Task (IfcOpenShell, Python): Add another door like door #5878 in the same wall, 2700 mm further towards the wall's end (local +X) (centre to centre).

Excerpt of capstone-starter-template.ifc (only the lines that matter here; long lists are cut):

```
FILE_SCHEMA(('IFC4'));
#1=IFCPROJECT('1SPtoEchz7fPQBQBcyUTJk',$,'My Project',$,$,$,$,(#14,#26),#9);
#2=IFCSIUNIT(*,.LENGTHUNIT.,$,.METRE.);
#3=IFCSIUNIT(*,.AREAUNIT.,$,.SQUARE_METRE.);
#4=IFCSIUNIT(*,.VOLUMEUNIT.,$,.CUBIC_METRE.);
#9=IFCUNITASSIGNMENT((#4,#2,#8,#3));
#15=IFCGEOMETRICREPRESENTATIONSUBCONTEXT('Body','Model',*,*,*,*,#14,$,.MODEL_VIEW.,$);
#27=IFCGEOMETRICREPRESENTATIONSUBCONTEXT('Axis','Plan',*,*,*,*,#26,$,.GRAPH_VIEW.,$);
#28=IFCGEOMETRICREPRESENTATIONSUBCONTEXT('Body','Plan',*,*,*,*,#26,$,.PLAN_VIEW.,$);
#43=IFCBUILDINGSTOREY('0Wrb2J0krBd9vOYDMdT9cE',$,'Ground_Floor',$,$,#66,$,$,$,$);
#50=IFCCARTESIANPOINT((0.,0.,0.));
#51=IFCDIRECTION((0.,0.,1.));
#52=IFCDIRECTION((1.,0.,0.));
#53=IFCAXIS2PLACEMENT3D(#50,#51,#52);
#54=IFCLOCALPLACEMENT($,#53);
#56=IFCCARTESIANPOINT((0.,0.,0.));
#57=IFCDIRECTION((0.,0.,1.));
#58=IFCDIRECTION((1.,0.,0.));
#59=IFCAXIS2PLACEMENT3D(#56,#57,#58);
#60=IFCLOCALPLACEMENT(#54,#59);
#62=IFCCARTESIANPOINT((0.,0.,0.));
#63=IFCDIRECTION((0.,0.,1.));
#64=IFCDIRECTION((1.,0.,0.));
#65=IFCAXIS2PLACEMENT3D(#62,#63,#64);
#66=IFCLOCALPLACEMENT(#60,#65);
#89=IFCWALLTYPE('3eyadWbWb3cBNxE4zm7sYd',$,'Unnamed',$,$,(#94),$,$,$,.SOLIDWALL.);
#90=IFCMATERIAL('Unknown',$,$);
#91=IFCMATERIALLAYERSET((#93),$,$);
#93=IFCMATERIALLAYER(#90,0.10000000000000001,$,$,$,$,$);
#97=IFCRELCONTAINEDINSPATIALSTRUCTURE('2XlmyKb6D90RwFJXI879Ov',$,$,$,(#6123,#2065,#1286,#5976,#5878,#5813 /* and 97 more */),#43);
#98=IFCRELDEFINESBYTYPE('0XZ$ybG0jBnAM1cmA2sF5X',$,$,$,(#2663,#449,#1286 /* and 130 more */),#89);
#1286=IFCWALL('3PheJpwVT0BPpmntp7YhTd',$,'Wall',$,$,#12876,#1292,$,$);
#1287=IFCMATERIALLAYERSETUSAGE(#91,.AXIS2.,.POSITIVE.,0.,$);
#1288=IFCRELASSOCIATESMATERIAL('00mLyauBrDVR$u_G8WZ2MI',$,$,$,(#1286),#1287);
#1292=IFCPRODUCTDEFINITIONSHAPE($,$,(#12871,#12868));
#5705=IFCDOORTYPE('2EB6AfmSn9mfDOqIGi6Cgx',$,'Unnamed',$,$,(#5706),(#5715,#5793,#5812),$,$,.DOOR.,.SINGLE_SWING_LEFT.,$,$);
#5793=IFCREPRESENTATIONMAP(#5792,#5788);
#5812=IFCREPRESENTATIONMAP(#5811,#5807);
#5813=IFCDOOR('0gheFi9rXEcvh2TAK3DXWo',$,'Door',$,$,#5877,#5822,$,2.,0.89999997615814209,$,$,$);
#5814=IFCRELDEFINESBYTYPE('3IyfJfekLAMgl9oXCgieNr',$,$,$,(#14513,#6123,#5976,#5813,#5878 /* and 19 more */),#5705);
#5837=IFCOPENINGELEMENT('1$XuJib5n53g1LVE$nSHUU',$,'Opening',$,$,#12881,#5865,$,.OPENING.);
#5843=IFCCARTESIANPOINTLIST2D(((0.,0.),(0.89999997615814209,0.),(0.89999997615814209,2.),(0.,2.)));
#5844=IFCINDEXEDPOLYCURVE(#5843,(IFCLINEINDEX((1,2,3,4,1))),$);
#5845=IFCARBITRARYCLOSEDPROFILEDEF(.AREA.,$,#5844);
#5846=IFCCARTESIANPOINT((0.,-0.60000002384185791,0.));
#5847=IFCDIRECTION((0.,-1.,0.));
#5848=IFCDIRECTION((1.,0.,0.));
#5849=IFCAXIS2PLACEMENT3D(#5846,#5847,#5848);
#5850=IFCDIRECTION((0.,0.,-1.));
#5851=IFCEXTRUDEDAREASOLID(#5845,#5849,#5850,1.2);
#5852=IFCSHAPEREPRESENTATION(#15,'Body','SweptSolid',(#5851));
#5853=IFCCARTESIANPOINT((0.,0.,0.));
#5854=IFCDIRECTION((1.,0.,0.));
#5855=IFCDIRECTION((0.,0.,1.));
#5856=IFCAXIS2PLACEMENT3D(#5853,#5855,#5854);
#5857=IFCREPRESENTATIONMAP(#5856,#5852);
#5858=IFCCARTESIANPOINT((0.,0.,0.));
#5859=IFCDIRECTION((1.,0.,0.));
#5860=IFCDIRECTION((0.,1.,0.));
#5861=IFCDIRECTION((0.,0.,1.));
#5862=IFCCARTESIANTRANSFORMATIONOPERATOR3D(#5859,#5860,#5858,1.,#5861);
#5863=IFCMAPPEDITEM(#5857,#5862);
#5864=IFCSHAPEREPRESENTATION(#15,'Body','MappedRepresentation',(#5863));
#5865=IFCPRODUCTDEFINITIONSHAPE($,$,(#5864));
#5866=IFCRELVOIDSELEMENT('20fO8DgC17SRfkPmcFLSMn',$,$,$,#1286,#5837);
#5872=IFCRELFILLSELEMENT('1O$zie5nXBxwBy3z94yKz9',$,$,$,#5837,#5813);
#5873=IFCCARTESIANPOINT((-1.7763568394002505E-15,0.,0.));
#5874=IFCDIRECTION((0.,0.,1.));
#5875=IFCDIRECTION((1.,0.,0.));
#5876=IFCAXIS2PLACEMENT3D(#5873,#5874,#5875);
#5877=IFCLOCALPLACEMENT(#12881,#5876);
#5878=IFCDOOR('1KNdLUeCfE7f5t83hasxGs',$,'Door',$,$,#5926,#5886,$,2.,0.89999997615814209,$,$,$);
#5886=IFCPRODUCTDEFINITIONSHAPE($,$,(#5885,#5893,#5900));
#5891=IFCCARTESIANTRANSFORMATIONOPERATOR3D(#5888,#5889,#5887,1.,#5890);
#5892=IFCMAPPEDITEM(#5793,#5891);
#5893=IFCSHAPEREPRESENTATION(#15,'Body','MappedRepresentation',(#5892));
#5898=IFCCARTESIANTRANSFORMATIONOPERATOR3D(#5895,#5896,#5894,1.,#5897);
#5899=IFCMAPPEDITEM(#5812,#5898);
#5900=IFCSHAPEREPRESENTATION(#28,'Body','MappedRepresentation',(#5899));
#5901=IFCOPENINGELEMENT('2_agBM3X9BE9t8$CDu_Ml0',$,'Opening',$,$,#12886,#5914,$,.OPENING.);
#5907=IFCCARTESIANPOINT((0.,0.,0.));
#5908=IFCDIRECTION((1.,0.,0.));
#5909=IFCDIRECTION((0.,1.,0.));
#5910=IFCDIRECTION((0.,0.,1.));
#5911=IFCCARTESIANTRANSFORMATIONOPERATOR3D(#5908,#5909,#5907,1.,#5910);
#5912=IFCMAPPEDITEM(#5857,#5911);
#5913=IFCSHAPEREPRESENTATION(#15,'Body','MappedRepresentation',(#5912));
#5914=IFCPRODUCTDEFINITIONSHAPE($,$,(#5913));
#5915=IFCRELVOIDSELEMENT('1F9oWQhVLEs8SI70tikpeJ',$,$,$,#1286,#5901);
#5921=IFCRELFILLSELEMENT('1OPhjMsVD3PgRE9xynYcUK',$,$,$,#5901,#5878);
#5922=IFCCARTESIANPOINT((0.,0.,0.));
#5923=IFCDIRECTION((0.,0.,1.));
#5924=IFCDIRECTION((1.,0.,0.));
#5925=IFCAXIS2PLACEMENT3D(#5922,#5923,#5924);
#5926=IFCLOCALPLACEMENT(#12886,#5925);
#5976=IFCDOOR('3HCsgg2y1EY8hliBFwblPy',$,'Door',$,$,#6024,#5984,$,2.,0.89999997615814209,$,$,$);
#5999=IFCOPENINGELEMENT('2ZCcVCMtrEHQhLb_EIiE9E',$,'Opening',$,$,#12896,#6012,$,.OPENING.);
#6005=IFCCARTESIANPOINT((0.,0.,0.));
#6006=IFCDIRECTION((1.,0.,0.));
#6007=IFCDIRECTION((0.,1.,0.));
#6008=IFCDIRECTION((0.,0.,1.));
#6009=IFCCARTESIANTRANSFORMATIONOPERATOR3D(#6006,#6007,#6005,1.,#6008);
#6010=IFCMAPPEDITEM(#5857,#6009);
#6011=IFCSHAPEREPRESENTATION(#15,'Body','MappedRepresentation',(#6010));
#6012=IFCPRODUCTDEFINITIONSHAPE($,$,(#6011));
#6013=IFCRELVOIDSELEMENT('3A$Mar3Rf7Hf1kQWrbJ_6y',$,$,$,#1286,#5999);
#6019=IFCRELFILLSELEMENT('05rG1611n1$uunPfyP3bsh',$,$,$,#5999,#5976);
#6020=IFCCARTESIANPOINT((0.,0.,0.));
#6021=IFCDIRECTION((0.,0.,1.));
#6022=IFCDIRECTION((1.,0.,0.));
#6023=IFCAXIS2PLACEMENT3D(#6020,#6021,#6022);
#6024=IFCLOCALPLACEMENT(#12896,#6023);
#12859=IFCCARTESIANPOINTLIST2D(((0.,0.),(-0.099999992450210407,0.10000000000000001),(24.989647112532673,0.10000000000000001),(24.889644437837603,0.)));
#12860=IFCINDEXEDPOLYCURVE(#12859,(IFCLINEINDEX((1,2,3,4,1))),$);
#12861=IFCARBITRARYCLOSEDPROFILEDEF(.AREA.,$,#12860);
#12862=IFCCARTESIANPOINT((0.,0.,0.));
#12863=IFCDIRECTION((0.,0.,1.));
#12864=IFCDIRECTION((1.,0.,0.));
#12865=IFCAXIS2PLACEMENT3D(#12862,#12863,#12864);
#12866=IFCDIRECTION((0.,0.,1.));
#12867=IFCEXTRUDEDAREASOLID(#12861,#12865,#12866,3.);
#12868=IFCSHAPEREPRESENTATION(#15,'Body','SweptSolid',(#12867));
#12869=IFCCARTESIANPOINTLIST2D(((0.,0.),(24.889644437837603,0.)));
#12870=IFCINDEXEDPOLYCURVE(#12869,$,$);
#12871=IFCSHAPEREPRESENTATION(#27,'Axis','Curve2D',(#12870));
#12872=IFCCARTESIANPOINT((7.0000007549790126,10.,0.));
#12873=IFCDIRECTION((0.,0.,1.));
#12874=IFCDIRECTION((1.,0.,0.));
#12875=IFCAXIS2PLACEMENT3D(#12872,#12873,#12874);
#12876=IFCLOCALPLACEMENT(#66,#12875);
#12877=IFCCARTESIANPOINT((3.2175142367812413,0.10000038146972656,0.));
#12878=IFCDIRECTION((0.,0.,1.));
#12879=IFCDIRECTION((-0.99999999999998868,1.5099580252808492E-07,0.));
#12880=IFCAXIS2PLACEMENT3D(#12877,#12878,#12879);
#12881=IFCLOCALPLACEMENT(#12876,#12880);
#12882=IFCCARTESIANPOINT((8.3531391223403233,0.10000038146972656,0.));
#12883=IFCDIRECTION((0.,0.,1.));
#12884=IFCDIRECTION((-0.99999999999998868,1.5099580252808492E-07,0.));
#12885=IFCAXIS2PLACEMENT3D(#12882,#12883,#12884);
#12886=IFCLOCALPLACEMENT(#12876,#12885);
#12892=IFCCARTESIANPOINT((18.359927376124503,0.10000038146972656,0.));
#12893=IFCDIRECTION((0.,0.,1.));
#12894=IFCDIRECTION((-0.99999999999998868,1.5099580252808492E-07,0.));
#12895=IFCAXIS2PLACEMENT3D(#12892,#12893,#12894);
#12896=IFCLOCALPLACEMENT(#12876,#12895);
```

```python
import ifcopenshell
import ifcopenshell.api.feature
import ifcopenshell.api.geometry
import ifcopenshell.api.root
import ifcopenshell.geom
import ifcopenshell.util.element
import ifcopenshell.util.placement
import ifcopenshell.util.shape
import ifcopenshell.util.unit

model = ifcopenshell.open("capstone-starter-template.ifc")
unit_scale = ifcopenshell.util.unit.calculate_unit_scale(model)
settings = ifcopenshell.geom.settings()


def volume(element):
    """Net volume in cubic metres, openings subtracted."""
    shape = ifcopenshell.geom.create_shape(settings, element)
    return ifcopenshell.util.shape.get_volume(shape.geometry)


door = model.by_id(5878)
opening = door.FillsVoids[0].RelatingOpeningElement
wall = opening.VoidsElements[0].RelatingBuildingElement
before = volume(wall)
shift = ifcopenshell.util.placement.get_local_placement(wall.ObjectPlacement)[:3, 0] * 2.7 / unit_scale

# copy_class copies the void relationship, type, container and properties, but no geometry.
new_opening = ifcopenshell.api.root.copy_class(model, product=opening)
new_opening.Representation = ifcopenshell.util.element.copy_deep(
    model, opening.Representation, exclude=["IfcGeometricRepresentationContext", "IfcRepresentationMap"]
)
new_door = ifcopenshell.api.root.copy_class(model, product=door)
new_door.Representation = ifcopenshell.util.element.copy_deep(
    model, door.Representation, exclude=["IfcGeometricRepresentationContext", "IfcRepresentationMap"]
)
ifcopenshell.api.feature.add_filling(model, opening=new_opening, element=new_door)

for old, new in ((opening, new_opening), (door, new_door)):
    matrix = ifcopenshell.util.placement.get_local_placement(old.ObjectPlacement)
    matrix[:3, 3] += shift
    ifcopenshell.api.geometry.edit_object_placement(model, product=new, matrix=matrix, is_si=False)

after = volume(wall)

print(f"wall volume {before:.3f} -> {after:.3f} m3")

model.write("capstone-starter-template_updated.ifc")
```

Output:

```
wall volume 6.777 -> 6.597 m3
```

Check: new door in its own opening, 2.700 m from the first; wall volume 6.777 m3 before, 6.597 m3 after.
